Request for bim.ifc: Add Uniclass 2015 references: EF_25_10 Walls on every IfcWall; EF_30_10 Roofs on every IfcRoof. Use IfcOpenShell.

First a look at what the model holds.

```python
import ifcopenshell

model = ifcopenshell.open("bim.ifc")
print(model.schema)
print("classifications:", [c.Name for c in model.by_type("IfcClassification")])
for ifc_class in ("IfcDoor", "IfcRoof", "IfcStair", "IfcWall", "IfcWindow"):
    print(ifc_class, len(model.by_type(ifc_class)))
```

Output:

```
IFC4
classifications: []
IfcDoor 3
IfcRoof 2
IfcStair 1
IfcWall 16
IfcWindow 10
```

```python
import ifcopenshell
import ifcopenshell.api.classification

model = ifcopenshell.open("bim.ifc")

system = ifcopenshell.api.classification.add_classification(model, classification="Uniclass 2015")

codes = {
    "IfcWall": ("EF_25_10", "Walls"),
    "IfcRoof": ("EF_30_10", "Roofs"),
}
for ifc_class, (code, name) in codes.items():
    products = model.by_type(ifc_class)
    ifcopenshell.api.classification.add_reference(
        model, products=products, classification=system, identification=code, name=name
    )
    print(code, len(products))

model.write("bim_rev.ifc")
```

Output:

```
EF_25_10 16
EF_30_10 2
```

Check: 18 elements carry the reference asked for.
